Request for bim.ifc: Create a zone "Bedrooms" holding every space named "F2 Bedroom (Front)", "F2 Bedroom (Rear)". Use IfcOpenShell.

First a look at what the model holds.

```python
import ifcopenshell

model = ifcopenshell.open("bim.ifc")
print(model.schema)
seen = {}
for space in model.by_type("IfcSpace"):
    seen[space.Name] = seen.get(space.Name, 0) + 1
for name, count in sorted(seen.items(), key=str):
    print(count, "x", name)
print("zones:", [z.Name for z in model.by_type("IfcZone")][:20])
```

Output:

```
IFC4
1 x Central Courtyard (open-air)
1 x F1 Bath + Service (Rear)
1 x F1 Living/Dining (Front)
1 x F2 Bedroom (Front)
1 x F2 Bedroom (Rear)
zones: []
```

```python
import ifcopenshell
import ifcopenshell.api.group
import ifcopenshell.api.root

model = ifcopenshell.open("bim.ifc")

names = {"F2 Bedroom (Front)", "F2 Bedroom (Rear)"}
spaces = [s for s in model.by_type("IfcSpace") if s.Name in names]

zone = ifcopenshell.api.root.create_entity(model, ifc_class="IfcZone", name="Bedrooms")
ifcopenshell.api.group.assign_group(model, products=spaces, group=zone)
print(len(spaces), "spaces in", zone.Name)

model.write("bim_rev.ifc")
```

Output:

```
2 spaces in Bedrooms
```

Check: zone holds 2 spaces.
